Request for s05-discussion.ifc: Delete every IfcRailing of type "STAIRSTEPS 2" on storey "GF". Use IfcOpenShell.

First a look at what the model holds.

```python
import ifcopenshell
import ifcopenshell.util.element

model = ifcopenshell.open("s05-discussion.ifc")
print(model.schema)
storey = next(s for s in model.by_type("IfcBuildingStorey") if s.Name == "GF")
railings = [e for e in ifcopenshell.util.element.get_decomposition(storey) if e.is_a("IfcRailing")]
seen = {}
for e in railings:
    element_type = ifcopenshell.util.element.get_type(e)
    name = element_type.Name if element_type not in (None, e) else None
    seen[name] = seen.get(name, 0) + 1
for name, count in sorted(seen.items(), key=str):
    print(count, "x", name)
```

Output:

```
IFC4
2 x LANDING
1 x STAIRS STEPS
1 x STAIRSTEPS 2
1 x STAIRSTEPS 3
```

```python
import ifcopenshell
import ifcopenshell.api.root
import ifcopenshell.util.element

model = ifcopenshell.open("s05-discussion.ifc")

storey = next(s for s in model.by_type("IfcBuildingStorey") if s.Name == "GF")
railings = [e for e in ifcopenshell.util.element.get_decomposition(storey) if e.is_a("IfcRailing")]
targets = [e for e in railings if (t := ifcopenshell.util.element.get_type(e)) not in (None, e) and t.Name == "STAIRSTEPS 2"]

for e in targets:
    ifcopenshell.api.root.remove_product(model, product=e)
print(len(targets), "removed")

model.write("s05-discussion_edited.ifc")
```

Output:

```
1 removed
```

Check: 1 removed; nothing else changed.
